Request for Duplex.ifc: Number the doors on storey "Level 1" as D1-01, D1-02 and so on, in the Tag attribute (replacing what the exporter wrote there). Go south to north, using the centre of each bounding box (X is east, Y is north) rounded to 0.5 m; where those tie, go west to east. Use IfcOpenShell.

First a look at what the model holds.

```python
import ifcopenshell
import ifcopenshell.util.element
import ifcopenshell.util.placement

model = ifcopenshell.open("Duplex.ifc")
print(model.schema)
storey = next(s for s in model.by_type("IfcBuildingStorey") if s.Name == "Level 1")
doors = [e for e in ifcopenshell.util.element.get_decomposition(storey) if e.is_a("IfcDoor")]
for e in sorted(doors, key=lambda e: e.id()):
    origin = ifcopenshell.util.placement.get_local_placement(e.ObjectPlacement)[:3, 3]
    print(e.id(), e.Tag, e.Name, origin.round(2) + 0.0, sep=" | ")
```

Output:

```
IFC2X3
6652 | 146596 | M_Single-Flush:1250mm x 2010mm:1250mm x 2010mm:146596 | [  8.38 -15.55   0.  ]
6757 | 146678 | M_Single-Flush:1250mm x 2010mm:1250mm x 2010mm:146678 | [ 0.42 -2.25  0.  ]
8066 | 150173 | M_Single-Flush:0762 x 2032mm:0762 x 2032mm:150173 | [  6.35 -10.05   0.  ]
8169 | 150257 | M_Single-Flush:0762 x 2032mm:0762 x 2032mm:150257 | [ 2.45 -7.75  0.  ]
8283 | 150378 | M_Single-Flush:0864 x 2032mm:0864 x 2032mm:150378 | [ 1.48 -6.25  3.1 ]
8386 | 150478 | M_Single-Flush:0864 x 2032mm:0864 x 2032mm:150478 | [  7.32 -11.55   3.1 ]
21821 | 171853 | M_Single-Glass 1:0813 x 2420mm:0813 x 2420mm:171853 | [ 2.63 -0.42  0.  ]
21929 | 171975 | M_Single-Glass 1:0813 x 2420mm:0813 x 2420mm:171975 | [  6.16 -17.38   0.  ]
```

```python
import ifcopenshell
import ifcopenshell.geom
import ifcopenshell.util.element
import ifcopenshell.util.shape

model = ifcopenshell.open("Duplex.ifc")
settings = ifcopenshell.geom.settings()
settings.set("use-world-coords", True)


def centre(element):
    shape = ifcopenshell.geom.create_shape(settings, element)
    return ifcopenshell.util.shape.get_bbox_centroid(shape.geometry)


storey = next(s for s in model.by_type("IfcBuildingStorey") if s.Name == "Level 1")
doors = [e for e in ifcopenshell.util.element.get_decomposition(storey) if e.is_a("IfcDoor")]

# Insertion points can sit at a corner or the storey origin, so sort by the geometry (in metres).
centres = {e: centre(e) for e in doors}
doors.sort(key=lambda e: (round(centres[e][1] / 0.5), centres[e][0]))

for i, e in enumerate(doors, start=1):
    number = f"D1-{i:02d}"
    e.Tag = number
    print(e.id(), number)

model.write("Duplex_edited.ifc")
```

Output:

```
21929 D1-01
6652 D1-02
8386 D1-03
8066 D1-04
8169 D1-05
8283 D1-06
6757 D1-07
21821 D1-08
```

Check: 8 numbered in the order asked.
